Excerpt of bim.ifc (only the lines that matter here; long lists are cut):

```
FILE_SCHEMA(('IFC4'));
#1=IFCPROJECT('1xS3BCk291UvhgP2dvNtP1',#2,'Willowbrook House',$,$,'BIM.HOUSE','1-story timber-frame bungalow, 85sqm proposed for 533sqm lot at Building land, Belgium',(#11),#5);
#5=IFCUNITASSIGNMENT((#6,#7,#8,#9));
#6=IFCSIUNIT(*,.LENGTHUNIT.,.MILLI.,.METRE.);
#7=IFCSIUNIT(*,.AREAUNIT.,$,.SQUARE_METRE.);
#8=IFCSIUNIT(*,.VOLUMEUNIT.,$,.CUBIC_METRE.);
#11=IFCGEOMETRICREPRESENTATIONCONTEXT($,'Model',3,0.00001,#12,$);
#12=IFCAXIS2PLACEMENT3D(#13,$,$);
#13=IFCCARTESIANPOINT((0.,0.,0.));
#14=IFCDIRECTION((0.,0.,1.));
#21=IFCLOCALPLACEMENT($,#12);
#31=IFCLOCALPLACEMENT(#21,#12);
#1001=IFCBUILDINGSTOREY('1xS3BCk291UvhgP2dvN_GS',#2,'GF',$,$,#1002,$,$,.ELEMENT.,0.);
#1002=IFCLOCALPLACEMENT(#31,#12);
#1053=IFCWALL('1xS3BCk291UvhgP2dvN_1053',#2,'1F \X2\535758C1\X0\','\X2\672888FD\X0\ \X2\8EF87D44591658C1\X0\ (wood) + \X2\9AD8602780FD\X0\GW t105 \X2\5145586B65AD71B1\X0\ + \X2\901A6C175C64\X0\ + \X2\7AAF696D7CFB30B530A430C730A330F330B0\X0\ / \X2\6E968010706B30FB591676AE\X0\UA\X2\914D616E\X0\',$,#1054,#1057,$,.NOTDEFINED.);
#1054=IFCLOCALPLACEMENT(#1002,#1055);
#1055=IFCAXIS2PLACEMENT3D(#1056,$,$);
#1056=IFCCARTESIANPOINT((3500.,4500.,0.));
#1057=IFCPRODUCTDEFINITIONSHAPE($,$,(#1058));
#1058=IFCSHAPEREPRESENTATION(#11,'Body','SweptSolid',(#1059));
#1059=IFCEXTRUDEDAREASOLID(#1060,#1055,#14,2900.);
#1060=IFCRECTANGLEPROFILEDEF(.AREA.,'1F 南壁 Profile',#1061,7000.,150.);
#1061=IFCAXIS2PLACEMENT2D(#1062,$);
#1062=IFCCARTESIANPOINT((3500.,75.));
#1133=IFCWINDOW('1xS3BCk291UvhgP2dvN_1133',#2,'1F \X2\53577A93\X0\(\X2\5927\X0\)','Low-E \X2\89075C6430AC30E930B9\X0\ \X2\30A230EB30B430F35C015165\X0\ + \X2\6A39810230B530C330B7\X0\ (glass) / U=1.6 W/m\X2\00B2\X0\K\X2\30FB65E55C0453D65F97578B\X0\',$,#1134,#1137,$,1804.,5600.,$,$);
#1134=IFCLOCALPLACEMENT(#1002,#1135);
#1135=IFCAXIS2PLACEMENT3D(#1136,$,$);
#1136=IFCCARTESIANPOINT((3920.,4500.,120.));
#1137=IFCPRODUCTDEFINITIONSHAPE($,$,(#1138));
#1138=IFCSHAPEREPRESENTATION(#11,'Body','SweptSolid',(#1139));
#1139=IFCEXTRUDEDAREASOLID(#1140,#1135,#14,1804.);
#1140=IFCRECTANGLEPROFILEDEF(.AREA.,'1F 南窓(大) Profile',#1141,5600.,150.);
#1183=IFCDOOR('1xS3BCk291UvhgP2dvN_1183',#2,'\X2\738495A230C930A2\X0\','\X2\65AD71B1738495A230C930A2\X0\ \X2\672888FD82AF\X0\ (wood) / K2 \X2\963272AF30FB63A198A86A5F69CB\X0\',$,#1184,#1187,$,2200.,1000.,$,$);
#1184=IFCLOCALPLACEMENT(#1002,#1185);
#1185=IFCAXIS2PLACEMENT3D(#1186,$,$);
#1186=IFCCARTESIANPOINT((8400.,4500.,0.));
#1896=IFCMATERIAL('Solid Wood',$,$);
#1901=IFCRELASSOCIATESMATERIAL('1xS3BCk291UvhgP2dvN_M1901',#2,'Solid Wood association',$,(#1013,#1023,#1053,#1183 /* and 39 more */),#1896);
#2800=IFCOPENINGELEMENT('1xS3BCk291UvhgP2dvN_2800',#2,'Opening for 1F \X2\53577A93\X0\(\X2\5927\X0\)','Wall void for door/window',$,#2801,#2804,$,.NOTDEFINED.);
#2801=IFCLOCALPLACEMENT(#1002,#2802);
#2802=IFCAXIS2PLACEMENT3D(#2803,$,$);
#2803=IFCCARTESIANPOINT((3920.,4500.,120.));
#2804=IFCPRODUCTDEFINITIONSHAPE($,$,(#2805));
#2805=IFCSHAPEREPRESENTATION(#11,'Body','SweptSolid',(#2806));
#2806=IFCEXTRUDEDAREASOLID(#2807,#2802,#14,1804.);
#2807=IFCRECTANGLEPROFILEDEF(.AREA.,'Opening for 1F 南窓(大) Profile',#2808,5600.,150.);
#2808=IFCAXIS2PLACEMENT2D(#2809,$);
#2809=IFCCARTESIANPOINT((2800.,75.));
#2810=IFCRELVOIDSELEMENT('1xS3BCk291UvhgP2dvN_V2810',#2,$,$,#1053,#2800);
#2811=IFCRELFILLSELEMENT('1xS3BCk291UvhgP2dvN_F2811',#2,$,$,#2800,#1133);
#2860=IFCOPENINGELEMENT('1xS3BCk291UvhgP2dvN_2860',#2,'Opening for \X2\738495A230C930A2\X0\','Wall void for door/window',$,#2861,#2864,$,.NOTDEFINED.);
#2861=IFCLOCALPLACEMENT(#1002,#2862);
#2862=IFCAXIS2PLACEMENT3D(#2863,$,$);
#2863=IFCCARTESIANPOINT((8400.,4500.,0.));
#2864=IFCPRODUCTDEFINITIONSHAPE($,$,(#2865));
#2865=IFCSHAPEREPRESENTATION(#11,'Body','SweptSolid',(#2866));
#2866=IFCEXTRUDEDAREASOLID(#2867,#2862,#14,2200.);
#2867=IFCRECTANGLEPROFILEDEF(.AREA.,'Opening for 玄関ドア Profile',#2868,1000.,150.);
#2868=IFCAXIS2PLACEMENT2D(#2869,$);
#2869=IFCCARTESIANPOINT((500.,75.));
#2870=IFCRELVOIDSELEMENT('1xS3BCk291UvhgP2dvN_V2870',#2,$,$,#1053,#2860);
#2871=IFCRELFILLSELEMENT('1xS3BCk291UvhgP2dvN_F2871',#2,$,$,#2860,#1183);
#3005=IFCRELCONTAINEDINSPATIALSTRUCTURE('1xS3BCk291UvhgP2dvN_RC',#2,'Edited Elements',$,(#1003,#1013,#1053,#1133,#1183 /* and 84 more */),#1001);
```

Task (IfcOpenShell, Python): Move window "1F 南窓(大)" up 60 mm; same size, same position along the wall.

```python
import numpy as np
import ifcopenshell
import ifcopenshell.api.geometry
import ifcopenshell.util.placement
import ifcopenshell.util.unit

model = ifcopenshell.open("bim.ifc")
unit_scale = ifcopenshell.util.unit.calculate_unit_scale(model)

window = model.by_guid("1xS3BCk291UvhgP2dvN_1133")
opening = window.FillsVoids[0].RelatingOpeningElement
dz = 0.06 / unit_scale

shift = np.array([0.0, 0.0, dz])
# The window is not placed relative to its opening, so move both.
for product in (opening, window):
    matrix = ifcopenshell.util.placement.get_local_placement(product.ObjectPlacement)
    matrix[:3, 3] += shift
    ifcopenshell.api.geometry.edit_object_placement(model, product=product, matrix=matrix, is_si=False)

print(f"moved by {dz * unit_scale:+.3f} m")

model.write("bim_rev.ifc")
```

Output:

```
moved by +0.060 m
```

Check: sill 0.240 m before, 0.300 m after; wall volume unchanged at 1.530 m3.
